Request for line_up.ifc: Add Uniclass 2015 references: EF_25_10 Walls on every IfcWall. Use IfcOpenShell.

First a look at what the model holds.

```python
import ifcopenshell

model = ifcopenshell.open("line_up.ifc")
print(model.schema)
print("classifications:", [c.Name for c in model.by_type("IfcClassification")])
for ifc_class in ("IfcDoor", "IfcRoof", "IfcStair", "IfcWall", "IfcWindow"):
    print(ifc_class, len(model.by_type(ifc_class)))
```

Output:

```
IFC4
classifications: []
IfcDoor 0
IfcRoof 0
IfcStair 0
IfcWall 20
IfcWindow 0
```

```python
import ifcopenshell
import ifcopenshell.api.classification

model = ifcopenshell.open("line_up.ifc")

system = ifcopenshell.api.classification.add_classification(model, classification="Uniclass 2015")

codes = {
    "IfcWall": ("EF_25_10", "Walls"),
}
for ifc_class, (code, name) in codes.items():
    products = model.by_type(ifc_class)
    ifcopenshell.api.classification.add_reference(
        model, products=products, classification=system, identification=code, name=name
    )
    print(code, len(products))

model.write("line_up_v2.ifc")
```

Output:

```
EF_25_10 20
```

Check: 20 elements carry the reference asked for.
